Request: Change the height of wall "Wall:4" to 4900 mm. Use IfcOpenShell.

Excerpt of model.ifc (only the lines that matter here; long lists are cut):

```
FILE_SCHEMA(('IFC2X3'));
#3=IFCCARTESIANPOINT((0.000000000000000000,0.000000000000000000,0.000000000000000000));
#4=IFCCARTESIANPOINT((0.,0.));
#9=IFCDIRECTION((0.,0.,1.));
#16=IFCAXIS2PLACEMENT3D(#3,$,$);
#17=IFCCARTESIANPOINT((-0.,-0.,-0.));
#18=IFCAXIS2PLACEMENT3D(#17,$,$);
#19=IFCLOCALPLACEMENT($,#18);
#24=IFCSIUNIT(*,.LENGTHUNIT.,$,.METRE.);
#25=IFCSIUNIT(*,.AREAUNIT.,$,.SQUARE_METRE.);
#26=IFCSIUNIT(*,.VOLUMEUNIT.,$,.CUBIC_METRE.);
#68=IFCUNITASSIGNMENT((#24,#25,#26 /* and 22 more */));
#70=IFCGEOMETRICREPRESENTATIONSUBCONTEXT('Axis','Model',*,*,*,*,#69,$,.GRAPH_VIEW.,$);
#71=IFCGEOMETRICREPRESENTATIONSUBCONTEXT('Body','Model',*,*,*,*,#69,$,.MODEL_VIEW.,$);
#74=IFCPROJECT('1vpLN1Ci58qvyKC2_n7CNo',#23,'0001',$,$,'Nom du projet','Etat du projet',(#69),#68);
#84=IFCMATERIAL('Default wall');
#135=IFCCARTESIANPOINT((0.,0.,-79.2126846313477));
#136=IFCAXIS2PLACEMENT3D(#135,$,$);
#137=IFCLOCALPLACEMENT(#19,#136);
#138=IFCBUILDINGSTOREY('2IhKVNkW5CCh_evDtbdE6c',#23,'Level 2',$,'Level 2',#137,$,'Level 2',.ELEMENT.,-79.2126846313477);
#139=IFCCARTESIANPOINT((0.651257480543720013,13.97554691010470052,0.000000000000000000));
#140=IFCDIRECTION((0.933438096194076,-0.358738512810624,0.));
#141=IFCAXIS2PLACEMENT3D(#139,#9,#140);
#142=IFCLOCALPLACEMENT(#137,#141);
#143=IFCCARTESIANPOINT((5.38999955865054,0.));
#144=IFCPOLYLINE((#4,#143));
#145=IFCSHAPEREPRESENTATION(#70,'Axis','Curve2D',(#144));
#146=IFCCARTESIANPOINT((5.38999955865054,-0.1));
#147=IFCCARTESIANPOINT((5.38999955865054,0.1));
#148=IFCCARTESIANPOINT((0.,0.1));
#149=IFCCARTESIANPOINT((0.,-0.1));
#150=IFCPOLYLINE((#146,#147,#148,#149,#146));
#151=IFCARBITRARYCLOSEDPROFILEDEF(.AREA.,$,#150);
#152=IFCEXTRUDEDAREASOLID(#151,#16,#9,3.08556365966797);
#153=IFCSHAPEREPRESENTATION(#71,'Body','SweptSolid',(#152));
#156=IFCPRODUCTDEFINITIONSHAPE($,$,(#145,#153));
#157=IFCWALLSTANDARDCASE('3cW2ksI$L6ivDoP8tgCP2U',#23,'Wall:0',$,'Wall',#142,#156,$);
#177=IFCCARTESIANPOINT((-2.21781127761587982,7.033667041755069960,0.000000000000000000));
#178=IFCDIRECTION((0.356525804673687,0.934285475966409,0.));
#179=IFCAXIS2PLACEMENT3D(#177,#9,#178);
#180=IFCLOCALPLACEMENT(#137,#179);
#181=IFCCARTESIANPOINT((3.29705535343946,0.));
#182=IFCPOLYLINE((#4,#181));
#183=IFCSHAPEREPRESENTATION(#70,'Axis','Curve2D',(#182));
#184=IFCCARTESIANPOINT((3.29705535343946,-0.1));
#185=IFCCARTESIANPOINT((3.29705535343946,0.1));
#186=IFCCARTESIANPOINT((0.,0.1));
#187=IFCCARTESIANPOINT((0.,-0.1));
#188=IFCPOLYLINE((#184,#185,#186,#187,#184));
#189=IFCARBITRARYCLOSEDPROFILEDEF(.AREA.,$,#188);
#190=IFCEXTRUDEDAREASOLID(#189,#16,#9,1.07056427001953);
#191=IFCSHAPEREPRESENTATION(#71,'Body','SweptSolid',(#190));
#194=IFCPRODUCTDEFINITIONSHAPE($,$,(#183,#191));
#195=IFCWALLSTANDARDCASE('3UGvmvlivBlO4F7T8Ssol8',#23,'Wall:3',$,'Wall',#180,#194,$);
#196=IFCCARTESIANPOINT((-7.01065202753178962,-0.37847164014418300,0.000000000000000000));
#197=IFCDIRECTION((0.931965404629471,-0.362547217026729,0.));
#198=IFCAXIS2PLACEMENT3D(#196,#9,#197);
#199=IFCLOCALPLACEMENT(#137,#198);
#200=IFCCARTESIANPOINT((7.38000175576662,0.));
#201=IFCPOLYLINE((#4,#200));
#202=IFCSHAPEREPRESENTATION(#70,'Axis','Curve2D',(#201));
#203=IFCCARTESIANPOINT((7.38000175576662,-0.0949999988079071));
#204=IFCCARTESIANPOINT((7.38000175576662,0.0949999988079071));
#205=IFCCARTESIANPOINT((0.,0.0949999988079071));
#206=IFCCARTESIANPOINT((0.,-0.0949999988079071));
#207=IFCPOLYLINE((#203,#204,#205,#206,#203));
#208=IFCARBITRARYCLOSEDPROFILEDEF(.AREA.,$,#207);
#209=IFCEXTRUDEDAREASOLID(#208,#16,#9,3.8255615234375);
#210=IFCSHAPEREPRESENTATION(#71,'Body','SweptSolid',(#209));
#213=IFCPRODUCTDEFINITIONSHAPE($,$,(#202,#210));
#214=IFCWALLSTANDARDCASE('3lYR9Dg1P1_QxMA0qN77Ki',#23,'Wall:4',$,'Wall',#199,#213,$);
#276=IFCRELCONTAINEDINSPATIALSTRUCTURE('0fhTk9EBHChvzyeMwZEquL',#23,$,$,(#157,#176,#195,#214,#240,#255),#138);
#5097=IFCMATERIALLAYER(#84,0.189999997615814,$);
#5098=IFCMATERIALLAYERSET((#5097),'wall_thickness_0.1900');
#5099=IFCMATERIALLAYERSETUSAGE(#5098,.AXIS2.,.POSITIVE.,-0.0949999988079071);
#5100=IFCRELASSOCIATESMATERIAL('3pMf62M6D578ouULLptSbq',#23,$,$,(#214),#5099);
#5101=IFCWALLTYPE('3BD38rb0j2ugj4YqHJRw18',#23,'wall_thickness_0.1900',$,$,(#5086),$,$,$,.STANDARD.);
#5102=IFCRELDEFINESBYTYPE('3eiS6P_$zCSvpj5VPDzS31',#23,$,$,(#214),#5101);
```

```python
import ifcopenshell
import ifcopenshell.geom
import ifcopenshell.util.representation
import ifcopenshell.util.shape
import ifcopenshell.util.unit

model = ifcopenshell.open("model.ifc")
unit_scale = ifcopenshell.util.unit.calculate_unit_scale(model)
settings = ifcopenshell.geom.settings()


def volume(element):
    """Net volume in cubic metres, openings subtracted."""
    shape = ifcopenshell.geom.create_shape(settings, element)
    return ifcopenshell.util.shape.get_volume(shape.geometry)


wall = model.by_guid("3lYR9Dg1P1_QxMA0qN77Ki")
before = volume(wall)

body = ifcopenshell.util.representation.get_representation(wall, "Model", "Body")
solid = body.Items[0]
old_height = solid.Depth
solid.Depth = 4.9 / unit_scale
after = volume(wall)

print(f"height {old_height:g} -> {solid.Depth:g}, volume {before:.3f} -> {after:.3f} m3")

model.write("model-out.ifc")
```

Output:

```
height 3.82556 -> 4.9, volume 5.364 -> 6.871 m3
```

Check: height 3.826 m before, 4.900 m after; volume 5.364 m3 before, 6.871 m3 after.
